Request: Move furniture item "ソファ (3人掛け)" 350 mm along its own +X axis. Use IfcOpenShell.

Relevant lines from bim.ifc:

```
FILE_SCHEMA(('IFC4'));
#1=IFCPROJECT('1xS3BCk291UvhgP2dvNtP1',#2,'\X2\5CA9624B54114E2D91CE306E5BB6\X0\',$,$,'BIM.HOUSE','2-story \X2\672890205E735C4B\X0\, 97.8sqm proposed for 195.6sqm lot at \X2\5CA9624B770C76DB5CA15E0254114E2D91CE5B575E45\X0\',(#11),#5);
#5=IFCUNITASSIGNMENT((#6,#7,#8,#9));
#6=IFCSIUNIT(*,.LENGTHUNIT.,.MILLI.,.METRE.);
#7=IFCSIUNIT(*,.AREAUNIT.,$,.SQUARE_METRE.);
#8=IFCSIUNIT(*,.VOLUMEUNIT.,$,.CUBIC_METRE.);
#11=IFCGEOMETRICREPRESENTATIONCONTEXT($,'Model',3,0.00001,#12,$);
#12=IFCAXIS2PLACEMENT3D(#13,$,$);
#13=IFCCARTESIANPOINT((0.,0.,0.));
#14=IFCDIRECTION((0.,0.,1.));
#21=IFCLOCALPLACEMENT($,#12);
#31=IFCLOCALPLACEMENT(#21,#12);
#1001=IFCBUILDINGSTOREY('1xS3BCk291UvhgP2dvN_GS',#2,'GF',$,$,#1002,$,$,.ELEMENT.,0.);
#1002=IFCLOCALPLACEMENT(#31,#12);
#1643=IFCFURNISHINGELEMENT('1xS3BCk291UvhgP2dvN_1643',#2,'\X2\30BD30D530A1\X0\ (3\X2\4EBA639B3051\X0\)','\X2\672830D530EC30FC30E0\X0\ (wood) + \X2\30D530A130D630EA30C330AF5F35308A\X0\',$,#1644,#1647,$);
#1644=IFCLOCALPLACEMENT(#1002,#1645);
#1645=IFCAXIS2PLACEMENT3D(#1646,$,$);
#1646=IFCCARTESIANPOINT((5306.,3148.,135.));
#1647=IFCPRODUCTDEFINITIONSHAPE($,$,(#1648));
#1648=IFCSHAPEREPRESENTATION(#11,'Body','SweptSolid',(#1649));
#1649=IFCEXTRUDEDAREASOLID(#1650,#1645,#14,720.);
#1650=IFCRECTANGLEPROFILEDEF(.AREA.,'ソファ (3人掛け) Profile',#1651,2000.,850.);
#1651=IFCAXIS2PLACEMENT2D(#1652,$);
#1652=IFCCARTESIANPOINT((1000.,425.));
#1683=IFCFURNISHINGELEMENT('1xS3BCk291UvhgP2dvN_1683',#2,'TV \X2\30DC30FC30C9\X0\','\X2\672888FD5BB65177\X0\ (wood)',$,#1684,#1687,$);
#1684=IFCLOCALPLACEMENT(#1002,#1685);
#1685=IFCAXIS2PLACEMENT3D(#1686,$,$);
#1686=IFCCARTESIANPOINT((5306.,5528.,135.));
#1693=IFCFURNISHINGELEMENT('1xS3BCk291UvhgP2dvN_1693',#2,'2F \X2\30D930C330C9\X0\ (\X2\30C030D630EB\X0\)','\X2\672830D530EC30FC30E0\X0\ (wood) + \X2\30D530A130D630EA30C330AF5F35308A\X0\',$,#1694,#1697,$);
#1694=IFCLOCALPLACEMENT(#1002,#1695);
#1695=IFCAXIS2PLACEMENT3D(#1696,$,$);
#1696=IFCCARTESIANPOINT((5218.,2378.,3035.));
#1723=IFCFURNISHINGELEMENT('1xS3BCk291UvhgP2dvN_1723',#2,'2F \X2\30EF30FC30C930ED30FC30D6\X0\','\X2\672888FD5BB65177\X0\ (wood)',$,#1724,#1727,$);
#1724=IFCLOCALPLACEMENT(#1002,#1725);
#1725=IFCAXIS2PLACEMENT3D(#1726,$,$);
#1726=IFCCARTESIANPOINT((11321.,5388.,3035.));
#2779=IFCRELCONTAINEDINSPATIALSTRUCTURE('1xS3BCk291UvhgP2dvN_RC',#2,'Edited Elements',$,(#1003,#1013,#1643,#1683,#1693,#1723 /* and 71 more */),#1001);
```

```python
import ifcopenshell
import ifcopenshell.api.geometry
import ifcopenshell.util.placement

model = ifcopenshell.open("bim.ifc")

item = model.by_guid("1xS3BCk291UvhgP2dvN_1643")
matrix = ifcopenshell.util.placement.get_local_placement(item.ObjectPlacement)
matrix[:3, 3] += matrix[:3, 0] * 350.0
ifcopenshell.api.geometry.edit_object_placement(model, product=item, matrix=matrix, is_si=False)

print(ifcopenshell.util.placement.get_local_placement(item.ObjectPlacement).round(3) + 0.0)

model.write("bim_rev.ifc")
```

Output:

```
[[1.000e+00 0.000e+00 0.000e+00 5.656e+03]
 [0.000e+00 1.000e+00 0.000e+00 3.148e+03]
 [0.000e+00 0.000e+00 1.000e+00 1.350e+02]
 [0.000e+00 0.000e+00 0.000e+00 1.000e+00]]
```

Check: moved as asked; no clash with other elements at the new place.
